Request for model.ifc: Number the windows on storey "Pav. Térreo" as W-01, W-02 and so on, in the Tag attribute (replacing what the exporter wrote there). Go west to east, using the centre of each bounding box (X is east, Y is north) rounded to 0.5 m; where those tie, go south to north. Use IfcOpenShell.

First a look at what the model holds.

```python
import ifcopenshell
import ifcopenshell.util.element
import ifcopenshell.util.placement

model = ifcopenshell.open("model.ifc")
print(model.schema)
storey = next(s for s in model.by_type("IfcBuildingStorey") if s.Name == "Pav. Térreo")
windows = [e for e in ifcopenshell.util.element.get_decomposition(storey) if e.is_a("IfcWindow")]
for e in sorted(windows, key=lambda e: e.id()):
    origin = ifcopenshell.util.placement.get_local_placement(e.ObjectPlacement)[:3, 3]
    print(e.id(), e.Tag, e.Name, origin.round(2) + 0.0, sep=" | ")
```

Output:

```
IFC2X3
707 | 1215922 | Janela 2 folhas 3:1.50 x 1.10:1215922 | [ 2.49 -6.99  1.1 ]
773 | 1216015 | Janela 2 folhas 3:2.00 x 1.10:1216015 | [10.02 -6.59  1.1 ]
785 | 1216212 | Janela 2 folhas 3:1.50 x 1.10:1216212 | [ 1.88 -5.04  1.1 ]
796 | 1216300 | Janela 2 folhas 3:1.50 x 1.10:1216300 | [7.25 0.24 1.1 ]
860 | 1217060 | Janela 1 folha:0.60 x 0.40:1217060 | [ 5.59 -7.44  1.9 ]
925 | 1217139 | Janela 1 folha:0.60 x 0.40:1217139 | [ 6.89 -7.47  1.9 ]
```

```python
import ifcopenshell
import ifcopenshell.geom
import ifcopenshell.util.element
import ifcopenshell.util.shape

model = ifcopenshell.open("model.ifc")
settings = ifcopenshell.geom.settings()
settings.set("use-world-coords", True)


def centre(element):
    shape = ifcopenshell.geom.create_shape(settings, element)
    return ifcopenshell.util.shape.get_bbox_centroid(shape.geometry)


storey = next(s for s in model.by_type("IfcBuildingStorey") if s.Name == "Pav. Térreo")
windows = [e for e in ifcopenshell.util.element.get_decomposition(storey) if e.is_a("IfcWindow")]

# Insertion points can sit at a corner or the storey origin, so sort by the geometry (in metres).
centres = {e: centre(e) for e in windows}
windows.sort(key=lambda e: (round(centres[e][0] / 0.5), centres[e][1]))

for i, e in enumerate(windows, start=1):
    number = f"W-{i:02d}"
    e.Tag = number
    print(e.id(), number)

model.write("model_edited.ifc")
```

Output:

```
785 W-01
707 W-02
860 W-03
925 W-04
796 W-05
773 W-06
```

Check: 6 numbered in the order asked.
